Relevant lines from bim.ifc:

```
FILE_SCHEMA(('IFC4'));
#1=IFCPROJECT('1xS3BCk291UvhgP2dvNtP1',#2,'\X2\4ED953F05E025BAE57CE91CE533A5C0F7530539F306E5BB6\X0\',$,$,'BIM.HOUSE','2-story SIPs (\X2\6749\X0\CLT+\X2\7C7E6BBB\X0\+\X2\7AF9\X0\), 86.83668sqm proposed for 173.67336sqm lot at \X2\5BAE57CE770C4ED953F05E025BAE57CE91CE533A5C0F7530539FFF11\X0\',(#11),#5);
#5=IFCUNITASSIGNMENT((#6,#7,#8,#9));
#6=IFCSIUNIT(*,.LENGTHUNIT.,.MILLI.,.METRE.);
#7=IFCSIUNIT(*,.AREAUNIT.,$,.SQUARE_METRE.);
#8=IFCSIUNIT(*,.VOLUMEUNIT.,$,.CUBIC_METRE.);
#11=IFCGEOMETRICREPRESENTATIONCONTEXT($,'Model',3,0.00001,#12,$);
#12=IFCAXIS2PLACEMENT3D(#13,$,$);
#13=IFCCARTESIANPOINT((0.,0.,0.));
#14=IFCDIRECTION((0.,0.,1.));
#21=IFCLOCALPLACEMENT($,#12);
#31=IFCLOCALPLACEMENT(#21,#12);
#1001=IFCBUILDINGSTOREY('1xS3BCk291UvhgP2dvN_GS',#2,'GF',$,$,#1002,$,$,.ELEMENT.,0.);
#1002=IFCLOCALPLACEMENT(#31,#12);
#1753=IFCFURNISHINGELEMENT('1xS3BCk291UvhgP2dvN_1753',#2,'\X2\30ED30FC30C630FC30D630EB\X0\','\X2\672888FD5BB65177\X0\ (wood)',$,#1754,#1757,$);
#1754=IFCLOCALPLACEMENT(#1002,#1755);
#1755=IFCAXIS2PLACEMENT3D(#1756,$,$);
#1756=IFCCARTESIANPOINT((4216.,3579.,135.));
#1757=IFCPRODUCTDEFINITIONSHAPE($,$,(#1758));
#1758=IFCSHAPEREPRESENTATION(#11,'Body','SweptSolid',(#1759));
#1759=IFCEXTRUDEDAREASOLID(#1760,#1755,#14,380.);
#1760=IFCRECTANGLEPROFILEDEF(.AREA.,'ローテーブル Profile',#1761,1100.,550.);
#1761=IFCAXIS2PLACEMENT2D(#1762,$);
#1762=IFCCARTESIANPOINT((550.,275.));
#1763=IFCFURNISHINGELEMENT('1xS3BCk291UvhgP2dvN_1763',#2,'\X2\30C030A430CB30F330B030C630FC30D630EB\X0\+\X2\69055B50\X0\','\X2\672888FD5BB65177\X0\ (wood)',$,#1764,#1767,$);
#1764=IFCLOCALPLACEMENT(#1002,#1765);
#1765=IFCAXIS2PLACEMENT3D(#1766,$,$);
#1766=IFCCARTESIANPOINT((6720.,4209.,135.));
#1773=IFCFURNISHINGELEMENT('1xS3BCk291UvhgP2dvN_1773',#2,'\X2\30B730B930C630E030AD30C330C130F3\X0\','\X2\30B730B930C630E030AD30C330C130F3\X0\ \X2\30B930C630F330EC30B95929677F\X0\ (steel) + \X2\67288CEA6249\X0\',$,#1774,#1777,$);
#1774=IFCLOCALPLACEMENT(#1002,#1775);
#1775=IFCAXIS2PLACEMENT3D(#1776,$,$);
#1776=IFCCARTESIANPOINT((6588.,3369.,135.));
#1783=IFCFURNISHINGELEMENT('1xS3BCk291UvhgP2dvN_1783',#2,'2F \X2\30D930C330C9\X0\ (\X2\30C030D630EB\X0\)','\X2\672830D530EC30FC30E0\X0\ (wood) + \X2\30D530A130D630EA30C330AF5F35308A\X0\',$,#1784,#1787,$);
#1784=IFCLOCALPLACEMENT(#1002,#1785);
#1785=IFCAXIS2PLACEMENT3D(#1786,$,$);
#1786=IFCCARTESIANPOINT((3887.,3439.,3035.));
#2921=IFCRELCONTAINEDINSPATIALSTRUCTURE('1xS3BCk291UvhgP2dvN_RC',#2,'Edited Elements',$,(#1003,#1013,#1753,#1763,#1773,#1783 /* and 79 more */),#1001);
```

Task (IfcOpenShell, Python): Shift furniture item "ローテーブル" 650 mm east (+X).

```python
import ifcopenshell
import ifcopenshell.api.geometry
import ifcopenshell.util.placement
import ifcopenshell.util.unit

model = ifcopenshell.open("bim.ifc")
unit_scale = ifcopenshell.util.unit.calculate_unit_scale(model)

item = model.by_guid("1xS3BCk291UvhgP2dvN_1753")
matrix = ifcopenshell.util.placement.get_local_placement(item.ObjectPlacement)
matrix[0, 3] += 0.65 / unit_scale
ifcopenshell.api.geometry.edit_object_placement(model, product=item, matrix=matrix, is_si=False)

print(ifcopenshell.util.placement.get_local_placement(item.ObjectPlacement).round(3) + 0.0)

model.write("bim_rev.ifc")
```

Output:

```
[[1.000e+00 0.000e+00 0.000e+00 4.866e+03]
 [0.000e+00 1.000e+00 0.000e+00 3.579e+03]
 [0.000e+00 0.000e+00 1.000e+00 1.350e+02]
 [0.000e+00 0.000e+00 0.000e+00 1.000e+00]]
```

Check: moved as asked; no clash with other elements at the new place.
